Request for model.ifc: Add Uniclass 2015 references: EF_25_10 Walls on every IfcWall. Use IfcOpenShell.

First a look at what the model holds.

```python
import ifcopenshell

model = ifcopenshell.open("model.ifc")
print(model.schema)
print("classifications:", [c.Name for c in model.by_type("IfcClassification")])
for ifc_class in ("IfcDoor", "IfcRoof", "IfcStair", "IfcWall", "IfcWindow"):
    print(ifc_class, len(model.by_type(ifc_class)))
```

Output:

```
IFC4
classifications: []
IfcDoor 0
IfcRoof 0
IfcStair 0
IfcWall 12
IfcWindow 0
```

```python
import ifcopenshell
import ifcopenshell.api.classification

model = ifcopenshell.open("model.ifc")

system = ifcopenshell.api.classification.add_classification(model, classification="Uniclass 2015")

codes = {
    "IfcWall": ("EF_25_10", "Walls"),
}
for ifc_class, (code, name) in codes.items():
    products = model.by_type(ifc_class)
    ifcopenshell.api.classification.add_reference(
        model, products=products, classification=system, identification=code, name=name
    )
    print(code, len(products))

model.write("model-out.ifc")
```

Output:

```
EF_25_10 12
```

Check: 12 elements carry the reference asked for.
